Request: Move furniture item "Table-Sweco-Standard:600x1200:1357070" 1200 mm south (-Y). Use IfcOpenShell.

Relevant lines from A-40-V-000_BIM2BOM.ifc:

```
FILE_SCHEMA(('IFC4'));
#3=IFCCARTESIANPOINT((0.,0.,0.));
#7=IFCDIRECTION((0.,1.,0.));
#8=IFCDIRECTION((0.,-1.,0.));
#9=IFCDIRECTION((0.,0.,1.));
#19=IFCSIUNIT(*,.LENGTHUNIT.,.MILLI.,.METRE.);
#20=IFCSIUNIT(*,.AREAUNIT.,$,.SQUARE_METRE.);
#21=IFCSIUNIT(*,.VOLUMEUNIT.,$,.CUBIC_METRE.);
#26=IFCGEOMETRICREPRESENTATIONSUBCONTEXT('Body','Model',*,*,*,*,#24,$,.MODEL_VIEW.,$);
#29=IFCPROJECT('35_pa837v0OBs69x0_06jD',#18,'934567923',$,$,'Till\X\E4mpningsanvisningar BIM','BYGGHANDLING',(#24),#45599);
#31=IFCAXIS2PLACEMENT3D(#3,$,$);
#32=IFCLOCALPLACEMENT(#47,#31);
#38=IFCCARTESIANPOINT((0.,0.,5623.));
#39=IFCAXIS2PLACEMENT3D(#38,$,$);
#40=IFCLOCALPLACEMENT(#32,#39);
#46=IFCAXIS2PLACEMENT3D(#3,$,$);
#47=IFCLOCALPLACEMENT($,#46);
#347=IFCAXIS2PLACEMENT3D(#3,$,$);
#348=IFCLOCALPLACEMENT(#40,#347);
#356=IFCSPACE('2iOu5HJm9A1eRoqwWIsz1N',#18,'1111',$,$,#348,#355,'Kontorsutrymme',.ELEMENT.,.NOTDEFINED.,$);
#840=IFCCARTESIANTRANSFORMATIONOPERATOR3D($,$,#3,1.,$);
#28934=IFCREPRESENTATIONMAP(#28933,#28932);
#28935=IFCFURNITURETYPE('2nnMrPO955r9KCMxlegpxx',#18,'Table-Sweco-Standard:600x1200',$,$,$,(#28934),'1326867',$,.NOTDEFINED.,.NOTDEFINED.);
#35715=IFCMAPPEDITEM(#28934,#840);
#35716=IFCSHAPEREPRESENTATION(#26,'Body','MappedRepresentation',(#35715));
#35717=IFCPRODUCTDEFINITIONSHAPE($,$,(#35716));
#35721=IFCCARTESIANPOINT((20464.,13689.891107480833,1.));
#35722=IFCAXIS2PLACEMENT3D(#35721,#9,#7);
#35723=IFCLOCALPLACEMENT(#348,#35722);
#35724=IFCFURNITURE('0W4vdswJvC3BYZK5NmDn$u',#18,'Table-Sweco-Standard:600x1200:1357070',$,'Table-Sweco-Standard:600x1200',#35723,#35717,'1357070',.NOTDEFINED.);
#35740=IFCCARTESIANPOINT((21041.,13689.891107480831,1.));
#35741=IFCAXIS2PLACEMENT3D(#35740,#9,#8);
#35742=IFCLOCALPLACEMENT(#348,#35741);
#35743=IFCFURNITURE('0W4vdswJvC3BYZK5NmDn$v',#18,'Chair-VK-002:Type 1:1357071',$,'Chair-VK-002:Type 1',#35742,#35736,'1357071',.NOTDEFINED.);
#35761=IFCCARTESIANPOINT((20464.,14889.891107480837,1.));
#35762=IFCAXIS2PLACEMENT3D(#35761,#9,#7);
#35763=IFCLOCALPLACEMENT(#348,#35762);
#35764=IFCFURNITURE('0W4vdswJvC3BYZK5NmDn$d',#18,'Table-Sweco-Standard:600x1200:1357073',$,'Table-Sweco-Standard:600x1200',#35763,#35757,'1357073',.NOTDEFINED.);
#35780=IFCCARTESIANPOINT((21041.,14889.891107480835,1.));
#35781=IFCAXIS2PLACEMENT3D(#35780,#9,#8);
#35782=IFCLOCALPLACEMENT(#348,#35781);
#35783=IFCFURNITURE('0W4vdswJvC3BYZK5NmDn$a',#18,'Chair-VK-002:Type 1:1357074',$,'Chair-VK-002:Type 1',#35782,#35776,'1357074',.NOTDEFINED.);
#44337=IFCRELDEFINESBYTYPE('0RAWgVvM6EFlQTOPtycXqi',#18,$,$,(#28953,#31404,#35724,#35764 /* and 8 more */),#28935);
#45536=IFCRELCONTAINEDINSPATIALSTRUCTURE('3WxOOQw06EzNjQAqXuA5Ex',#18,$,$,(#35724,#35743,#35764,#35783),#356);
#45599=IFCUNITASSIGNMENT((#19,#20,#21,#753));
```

```python
import ifcopenshell
import ifcopenshell.api.geometry
import ifcopenshell.util.placement

model = ifcopenshell.open("A-40-V-000_BIM2BOM.ifc")

item = model.by_guid("0W4vdswJvC3BYZK5NmDn$u")
matrix = ifcopenshell.util.placement.get_local_placement(item.ObjectPlacement)
matrix[1, 3] -= 1200.0
ifcopenshell.api.geometry.edit_object_placement(model, product=item, matrix=matrix, is_si=False)

print(ifcopenshell.util.placement.get_local_placement(item.ObjectPlacement).round(3) + 0.0)

model.write("A-40-V-000_BIM2BOM_updated.ifc")
```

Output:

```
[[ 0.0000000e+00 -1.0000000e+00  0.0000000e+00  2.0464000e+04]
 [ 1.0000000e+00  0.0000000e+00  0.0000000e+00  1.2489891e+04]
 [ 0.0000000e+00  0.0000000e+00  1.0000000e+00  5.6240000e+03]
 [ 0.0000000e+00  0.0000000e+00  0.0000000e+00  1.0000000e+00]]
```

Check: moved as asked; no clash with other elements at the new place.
